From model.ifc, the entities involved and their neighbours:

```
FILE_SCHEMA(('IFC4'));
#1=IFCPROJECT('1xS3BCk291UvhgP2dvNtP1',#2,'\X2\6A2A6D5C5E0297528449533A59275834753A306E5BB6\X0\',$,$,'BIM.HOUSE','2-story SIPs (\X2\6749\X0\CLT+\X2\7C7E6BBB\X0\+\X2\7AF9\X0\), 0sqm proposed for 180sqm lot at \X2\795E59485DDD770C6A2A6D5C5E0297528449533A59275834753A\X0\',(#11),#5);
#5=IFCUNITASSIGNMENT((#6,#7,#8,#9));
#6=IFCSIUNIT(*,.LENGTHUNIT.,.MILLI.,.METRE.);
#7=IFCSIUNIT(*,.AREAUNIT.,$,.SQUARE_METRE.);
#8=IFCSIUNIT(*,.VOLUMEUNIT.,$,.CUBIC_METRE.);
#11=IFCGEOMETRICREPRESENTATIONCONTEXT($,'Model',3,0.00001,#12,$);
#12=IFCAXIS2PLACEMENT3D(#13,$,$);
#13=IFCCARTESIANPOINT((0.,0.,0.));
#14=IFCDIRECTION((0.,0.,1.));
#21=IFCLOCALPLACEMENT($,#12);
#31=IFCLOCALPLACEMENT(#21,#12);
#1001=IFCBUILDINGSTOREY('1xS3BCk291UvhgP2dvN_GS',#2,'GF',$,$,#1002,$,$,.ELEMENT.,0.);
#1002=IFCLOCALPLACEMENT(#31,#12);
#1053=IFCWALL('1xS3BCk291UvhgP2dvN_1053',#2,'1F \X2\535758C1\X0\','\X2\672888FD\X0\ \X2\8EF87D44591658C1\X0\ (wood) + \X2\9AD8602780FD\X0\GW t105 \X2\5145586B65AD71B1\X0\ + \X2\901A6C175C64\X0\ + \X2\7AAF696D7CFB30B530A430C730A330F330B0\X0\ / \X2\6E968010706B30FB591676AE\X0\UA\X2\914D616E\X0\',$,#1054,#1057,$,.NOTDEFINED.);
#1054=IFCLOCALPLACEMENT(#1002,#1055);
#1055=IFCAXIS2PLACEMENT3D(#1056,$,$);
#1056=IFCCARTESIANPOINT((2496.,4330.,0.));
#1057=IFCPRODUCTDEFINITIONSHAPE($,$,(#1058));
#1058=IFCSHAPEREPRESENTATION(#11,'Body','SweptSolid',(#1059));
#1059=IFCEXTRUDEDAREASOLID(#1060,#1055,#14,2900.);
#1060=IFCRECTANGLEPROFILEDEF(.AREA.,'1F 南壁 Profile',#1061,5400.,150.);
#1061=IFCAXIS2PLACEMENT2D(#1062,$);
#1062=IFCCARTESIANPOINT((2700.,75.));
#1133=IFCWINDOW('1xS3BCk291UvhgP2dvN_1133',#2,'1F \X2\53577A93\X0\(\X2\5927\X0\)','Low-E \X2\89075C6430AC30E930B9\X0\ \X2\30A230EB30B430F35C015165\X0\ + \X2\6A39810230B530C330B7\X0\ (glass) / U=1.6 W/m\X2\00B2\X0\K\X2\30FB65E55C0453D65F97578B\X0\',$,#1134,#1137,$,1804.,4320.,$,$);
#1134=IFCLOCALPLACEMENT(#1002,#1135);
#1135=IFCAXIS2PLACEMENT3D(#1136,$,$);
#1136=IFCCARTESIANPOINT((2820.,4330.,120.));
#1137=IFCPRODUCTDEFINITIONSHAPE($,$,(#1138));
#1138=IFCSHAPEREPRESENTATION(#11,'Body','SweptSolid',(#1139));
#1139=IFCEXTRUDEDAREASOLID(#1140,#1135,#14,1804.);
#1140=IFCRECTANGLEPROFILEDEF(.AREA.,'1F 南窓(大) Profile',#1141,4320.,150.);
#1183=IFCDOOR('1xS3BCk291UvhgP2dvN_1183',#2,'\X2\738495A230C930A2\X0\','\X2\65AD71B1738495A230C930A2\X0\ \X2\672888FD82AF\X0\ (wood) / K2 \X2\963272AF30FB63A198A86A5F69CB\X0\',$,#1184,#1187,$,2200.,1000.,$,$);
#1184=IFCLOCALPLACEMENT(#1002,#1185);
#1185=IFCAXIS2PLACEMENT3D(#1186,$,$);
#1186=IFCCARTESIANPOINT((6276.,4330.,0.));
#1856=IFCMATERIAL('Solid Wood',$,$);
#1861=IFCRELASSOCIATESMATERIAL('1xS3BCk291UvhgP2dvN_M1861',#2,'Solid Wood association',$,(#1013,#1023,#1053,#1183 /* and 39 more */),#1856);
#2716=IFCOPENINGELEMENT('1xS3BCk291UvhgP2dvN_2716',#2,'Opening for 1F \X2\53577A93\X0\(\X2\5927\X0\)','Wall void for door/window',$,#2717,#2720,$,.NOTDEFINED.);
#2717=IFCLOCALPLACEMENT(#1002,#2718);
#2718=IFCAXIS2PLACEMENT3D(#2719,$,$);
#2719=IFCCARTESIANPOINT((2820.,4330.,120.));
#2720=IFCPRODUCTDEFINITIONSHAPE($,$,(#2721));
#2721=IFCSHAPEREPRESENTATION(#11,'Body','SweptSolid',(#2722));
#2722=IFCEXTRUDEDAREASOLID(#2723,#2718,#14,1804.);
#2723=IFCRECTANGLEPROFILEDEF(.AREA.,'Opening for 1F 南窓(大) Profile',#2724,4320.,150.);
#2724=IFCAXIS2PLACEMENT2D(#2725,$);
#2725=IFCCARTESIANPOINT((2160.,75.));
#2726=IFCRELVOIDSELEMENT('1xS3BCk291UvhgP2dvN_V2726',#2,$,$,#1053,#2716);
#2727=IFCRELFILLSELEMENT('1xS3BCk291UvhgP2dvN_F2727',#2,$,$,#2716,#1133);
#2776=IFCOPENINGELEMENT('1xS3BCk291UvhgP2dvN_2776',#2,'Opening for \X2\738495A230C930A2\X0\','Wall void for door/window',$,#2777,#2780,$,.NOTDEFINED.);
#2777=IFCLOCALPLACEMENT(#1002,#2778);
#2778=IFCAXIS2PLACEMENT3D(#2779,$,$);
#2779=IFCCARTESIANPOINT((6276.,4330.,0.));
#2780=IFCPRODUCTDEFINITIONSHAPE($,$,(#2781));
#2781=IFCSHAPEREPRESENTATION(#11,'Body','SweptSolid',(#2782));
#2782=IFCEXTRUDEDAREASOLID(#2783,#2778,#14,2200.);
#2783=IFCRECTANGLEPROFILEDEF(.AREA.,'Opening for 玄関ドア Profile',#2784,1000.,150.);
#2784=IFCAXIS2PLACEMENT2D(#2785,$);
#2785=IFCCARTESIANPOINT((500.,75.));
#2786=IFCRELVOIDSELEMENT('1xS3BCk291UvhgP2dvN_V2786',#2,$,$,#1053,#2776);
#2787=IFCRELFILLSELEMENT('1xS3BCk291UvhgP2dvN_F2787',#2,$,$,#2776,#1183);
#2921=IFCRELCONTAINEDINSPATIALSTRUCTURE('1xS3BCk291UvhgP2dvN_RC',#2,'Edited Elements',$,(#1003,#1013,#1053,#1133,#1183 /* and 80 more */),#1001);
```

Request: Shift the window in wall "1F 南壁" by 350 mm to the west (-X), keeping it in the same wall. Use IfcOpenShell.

```python
import ifcopenshell
import ifcopenshell.api.geometry
import ifcopenshell.util.placement

model = ifcopenshell.open("model.ifc")

window = model.by_guid("1xS3BCk291UvhgP2dvN_1133")
opening = window.FillsVoids[0].RelatingOpeningElement
wall = opening.VoidsElements[0].RelatingBuildingElement

wall_matrix = ifcopenshell.util.placement.get_local_placement(wall.ObjectPlacement)
shift = wall_matrix[:3, 0] * -350.0
before = ifcopenshell.util.placement.get_local_placement(window.ObjectPlacement)[:3, 3].copy()

# The window is not placed relative to its opening, so move both.
for product in (opening, window):
    matrix = ifcopenshell.util.placement.get_local_placement(product.ObjectPlacement)
    matrix[:3, 3] += shift
    ifcopenshell.api.geometry.edit_object_placement(model, product=product, matrix=matrix, is_si=False)

after = ifcopenshell.util.placement.get_local_placement(window.ObjectPlacement)[:3, 3]
print("window moved by", (after - before).round(3) + 0.0)

model.write("model_edited.ifc")
```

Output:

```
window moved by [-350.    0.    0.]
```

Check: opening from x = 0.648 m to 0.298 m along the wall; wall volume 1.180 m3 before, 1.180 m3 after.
